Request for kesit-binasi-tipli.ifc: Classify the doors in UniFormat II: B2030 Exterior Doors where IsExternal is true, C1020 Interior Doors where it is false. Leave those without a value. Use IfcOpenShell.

First a look at what the model holds.

```python
import ifcopenshell
import ifcopenshell.util.element

model = ifcopenshell.open("kesit-binasi-tipli.ifc")
print(model.schema)
print("classifications:", [c.Name for c in model.by_type("IfcClassification")])
values = [ifcopenshell.util.element.get_pset(e, "Pset_DoorCommon", "IsExternal") for e in model.by_type("IfcDoor")]
for value in (True, False, None):
    print("IsExternal", value, values.count(value))
```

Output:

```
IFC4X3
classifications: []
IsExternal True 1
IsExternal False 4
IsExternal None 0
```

```python
import ifcopenshell
import ifcopenshell.api.classification
import ifcopenshell.util.element

model = ifcopenshell.open("kesit-binasi-tipli.ifc")

system = ifcopenshell.api.classification.add_classification(model, classification="UniFormat II")

doors = model.by_type("IfcDoor")
external = {e: ifcopenshell.util.element.get_pset(e, "Pset_DoorCommon", "IsExternal") for e in doors}
for flag, code, name in ((True, "B2030", "Exterior Doors"), (False, "C1020", "Interior Doors")):
    products = [e for e in doors if external[e] is flag]
    ifcopenshell.api.classification.add_reference(
        model, products=products, classification=system, identification=code, name=name
    )
    print(code, len(products))

model.write("kesit-binasi-tipli_edited.ifc")
```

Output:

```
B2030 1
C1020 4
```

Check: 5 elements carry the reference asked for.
